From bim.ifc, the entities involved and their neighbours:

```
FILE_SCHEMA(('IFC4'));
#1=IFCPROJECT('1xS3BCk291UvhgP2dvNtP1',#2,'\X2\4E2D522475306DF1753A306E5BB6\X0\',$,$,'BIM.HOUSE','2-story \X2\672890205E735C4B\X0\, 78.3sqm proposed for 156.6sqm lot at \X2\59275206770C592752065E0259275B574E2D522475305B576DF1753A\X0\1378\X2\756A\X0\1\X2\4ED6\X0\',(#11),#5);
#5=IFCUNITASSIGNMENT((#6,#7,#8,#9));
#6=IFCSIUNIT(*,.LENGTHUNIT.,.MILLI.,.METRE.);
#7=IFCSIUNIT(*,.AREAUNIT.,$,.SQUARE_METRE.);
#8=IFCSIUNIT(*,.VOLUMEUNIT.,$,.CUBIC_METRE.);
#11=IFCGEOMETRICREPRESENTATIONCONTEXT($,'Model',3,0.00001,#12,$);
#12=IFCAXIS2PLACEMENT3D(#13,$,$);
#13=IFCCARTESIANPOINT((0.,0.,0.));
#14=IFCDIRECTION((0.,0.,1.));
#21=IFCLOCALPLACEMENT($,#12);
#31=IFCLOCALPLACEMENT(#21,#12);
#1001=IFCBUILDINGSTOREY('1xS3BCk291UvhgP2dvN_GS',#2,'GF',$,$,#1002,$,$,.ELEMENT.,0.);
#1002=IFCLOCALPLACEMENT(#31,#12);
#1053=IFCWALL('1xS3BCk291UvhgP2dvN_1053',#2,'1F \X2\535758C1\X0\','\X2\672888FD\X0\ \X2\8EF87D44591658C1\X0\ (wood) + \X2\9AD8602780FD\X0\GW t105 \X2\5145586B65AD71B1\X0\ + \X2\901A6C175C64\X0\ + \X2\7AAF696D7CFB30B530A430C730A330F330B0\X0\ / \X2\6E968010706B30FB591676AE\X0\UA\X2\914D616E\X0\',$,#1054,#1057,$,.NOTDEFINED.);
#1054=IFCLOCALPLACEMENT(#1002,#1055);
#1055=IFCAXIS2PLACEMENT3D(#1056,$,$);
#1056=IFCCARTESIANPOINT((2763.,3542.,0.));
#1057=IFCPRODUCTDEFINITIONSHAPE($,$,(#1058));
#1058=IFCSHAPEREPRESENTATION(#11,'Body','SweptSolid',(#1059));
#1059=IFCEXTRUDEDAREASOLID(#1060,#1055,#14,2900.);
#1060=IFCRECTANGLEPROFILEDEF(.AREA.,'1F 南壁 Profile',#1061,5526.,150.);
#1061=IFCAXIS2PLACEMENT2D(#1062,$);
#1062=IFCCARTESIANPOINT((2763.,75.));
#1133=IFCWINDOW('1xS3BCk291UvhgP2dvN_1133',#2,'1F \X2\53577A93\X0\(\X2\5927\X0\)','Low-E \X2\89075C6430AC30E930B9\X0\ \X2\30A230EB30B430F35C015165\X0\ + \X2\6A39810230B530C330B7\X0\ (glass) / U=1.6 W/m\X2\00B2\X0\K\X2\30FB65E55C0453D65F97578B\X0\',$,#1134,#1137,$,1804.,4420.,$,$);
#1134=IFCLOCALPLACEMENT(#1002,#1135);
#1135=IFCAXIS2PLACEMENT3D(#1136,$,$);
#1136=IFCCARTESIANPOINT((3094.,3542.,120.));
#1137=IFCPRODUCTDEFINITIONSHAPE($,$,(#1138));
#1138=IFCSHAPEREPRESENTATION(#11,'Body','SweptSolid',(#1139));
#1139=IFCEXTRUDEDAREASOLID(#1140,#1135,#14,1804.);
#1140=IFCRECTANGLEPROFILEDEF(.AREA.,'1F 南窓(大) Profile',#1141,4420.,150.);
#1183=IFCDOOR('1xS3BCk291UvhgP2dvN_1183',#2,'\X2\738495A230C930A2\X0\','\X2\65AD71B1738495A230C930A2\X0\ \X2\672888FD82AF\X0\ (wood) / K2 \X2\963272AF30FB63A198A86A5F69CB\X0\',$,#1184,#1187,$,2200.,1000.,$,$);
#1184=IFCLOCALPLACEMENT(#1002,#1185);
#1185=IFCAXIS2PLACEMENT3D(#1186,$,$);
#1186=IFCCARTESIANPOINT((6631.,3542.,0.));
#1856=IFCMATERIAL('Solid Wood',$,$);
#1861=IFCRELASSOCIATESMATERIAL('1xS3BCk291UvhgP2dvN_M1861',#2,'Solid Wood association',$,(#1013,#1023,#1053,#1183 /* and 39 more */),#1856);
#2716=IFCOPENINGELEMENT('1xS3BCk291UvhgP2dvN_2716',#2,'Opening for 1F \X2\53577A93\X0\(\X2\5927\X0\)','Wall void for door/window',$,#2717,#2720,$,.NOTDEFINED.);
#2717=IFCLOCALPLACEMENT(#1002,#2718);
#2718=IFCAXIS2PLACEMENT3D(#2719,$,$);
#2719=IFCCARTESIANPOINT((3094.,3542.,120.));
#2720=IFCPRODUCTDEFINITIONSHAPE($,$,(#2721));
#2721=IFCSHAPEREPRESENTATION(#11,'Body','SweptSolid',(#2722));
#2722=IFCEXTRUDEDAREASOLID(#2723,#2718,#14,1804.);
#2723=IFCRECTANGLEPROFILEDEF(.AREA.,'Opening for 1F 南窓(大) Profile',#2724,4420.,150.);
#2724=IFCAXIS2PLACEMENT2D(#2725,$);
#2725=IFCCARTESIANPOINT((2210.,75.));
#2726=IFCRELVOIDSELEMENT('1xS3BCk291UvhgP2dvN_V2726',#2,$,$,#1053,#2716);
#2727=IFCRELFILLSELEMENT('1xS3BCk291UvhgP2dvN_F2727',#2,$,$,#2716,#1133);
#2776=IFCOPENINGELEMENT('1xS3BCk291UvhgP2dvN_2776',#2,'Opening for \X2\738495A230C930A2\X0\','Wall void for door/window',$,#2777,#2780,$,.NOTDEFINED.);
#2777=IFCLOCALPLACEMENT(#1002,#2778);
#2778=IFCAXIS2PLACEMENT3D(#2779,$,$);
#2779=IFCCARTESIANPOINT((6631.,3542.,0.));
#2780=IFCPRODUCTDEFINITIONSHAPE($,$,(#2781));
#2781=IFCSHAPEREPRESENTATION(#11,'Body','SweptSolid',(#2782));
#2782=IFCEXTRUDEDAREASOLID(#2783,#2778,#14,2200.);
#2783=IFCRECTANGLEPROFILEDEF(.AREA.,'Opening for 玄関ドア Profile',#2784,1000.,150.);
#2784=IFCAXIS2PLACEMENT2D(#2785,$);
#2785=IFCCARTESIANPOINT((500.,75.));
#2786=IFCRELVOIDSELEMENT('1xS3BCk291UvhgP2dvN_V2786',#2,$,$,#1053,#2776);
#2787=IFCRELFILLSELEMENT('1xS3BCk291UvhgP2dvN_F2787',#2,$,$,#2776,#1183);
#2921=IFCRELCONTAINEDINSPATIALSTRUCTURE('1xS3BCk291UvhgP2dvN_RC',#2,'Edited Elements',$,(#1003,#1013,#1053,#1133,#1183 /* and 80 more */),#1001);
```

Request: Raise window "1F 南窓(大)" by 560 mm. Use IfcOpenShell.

```python
import numpy as np
import ifcopenshell
import ifcopenshell.api.geometry
import ifcopenshell.util.placement
import ifcopenshell.util.unit

model = ifcopenshell.open("bim.ifc")
unit_scale = ifcopenshell.util.unit.calculate_unit_scale(model)

window = model.by_id(1133)
opening = window.FillsVoids[0].RelatingOpeningElement
dz = 560.0

shift = np.array([0.0, 0.0, dz])
# The window is not placed relative to its opening, so move both.
for product in (opening, window):
    matrix = ifcopenshell.util.placement.get_local_placement(product.ObjectPlacement)
    matrix[:3, 3] += shift
    ifcopenshell.api.geometry.edit_object_placement(model, product=product, matrix=matrix, is_si=False)

print(f"moved by {dz * unit_scale:+.3f} m")

model.write("bim_v2.ifc")
```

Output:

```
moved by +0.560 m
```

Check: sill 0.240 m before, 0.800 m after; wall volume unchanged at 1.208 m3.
